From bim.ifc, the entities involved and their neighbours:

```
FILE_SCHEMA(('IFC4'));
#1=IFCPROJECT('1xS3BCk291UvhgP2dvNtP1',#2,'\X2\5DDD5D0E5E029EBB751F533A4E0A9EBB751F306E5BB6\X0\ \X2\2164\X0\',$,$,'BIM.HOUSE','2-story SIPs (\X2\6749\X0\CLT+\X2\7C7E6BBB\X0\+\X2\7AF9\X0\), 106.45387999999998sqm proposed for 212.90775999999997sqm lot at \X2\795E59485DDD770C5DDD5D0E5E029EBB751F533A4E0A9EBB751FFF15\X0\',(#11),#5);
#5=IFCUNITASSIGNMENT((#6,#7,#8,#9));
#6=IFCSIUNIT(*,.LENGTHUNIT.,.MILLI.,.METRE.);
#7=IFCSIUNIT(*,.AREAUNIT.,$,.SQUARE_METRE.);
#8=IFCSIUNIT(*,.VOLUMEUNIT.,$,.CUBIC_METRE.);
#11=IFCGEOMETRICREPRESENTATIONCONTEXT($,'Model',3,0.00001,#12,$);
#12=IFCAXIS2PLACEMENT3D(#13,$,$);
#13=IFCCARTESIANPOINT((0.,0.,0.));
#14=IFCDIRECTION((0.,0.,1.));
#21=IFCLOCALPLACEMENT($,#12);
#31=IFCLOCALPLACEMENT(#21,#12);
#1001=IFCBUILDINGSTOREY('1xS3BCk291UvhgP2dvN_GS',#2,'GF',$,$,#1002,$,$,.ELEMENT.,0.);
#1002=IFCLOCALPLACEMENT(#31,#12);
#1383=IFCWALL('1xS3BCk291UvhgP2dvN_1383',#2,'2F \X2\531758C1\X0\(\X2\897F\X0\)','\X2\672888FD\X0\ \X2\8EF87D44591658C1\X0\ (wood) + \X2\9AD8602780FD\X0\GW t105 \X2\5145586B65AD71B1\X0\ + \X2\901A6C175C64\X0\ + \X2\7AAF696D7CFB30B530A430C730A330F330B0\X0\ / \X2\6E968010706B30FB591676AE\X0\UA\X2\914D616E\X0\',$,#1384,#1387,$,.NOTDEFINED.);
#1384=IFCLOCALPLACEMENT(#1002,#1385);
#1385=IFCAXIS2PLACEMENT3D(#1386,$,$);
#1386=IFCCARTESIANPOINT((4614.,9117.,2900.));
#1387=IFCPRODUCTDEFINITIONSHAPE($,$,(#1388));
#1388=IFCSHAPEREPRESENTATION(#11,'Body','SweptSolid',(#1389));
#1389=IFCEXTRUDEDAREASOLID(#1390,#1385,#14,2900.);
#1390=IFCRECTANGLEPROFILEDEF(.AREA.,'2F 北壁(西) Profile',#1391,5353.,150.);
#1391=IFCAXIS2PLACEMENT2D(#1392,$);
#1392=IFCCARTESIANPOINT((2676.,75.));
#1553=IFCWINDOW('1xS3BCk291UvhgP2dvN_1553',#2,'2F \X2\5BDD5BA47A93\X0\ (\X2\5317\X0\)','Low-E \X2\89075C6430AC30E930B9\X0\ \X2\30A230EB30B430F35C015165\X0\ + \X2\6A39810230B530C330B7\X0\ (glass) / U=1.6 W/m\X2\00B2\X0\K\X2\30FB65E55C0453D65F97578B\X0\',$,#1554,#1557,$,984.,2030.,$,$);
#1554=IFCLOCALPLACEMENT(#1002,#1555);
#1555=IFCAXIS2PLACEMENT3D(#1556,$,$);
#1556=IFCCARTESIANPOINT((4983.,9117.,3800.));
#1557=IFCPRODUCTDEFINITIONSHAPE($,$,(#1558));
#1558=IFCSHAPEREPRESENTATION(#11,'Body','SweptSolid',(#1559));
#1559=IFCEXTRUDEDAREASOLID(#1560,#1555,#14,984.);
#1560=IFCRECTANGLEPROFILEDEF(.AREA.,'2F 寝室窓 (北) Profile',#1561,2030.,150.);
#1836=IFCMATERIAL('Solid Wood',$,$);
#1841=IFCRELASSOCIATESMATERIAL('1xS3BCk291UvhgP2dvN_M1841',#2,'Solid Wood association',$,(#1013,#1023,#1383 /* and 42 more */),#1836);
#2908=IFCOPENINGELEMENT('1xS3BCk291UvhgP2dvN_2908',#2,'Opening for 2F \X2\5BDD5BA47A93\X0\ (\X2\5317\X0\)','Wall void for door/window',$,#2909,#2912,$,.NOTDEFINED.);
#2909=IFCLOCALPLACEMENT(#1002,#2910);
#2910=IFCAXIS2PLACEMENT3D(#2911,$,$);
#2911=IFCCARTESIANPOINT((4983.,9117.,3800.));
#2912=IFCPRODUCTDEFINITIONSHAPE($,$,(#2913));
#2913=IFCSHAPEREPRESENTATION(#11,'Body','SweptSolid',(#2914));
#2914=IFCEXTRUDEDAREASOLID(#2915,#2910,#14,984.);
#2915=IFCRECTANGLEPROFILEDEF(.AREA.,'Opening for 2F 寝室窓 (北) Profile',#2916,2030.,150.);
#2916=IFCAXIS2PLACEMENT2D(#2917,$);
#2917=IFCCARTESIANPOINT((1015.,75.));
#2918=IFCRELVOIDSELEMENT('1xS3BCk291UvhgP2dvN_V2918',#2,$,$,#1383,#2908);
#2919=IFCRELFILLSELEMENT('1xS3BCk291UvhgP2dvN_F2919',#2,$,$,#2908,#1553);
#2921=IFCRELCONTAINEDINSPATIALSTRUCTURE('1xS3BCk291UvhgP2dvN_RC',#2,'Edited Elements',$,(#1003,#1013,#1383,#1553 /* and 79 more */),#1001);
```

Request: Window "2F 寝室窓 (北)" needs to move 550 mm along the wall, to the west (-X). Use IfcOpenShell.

```python
import ifcopenshell
import ifcopenshell.api.geometry
import ifcopenshell.util.placement
import ifcopenshell.util.unit

model = ifcopenshell.open("bim.ifc")
unit_scale = ifcopenshell.util.unit.calculate_unit_scale(model)

window = model.by_guid("1xS3BCk291UvhgP2dvN_1553")
opening = window.FillsVoids[0].RelatingOpeningElement
wall = opening.VoidsElements[0].RelatingBuildingElement

wall_matrix = ifcopenshell.util.placement.get_local_placement(wall.ObjectPlacement)
shift = wall_matrix[:3, 0] * -0.55 / unit_scale
before = ifcopenshell.util.placement.get_local_placement(window.ObjectPlacement)[:3, 3].copy()

# The window is not placed relative to its opening, so move both.
for product in (opening, window):
    matrix = ifcopenshell.util.placement.get_local_placement(product.ObjectPlacement)
    matrix[:3, 3] += shift
    ifcopenshell.api.geometry.edit_object_placement(model, product=product, matrix=matrix, is_si=False)

after = ifcopenshell.util.placement.get_local_placement(window.ObjectPlacement)[:3, 3]
print("window moved by", (after - before).round(3) + 0.0)

model.write("bim_rev.ifc")
```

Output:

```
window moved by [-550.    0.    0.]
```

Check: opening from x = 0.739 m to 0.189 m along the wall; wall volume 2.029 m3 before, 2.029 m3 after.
